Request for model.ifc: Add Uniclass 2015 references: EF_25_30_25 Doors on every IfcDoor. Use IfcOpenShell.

First a look at what the model holds.

```python
import ifcopenshell

model = ifcopenshell.open("model.ifc")
print(model.schema)
print("classifications:", [c.Name for c in model.by_type("IfcClassification")])
for ifc_class in ("IfcDoor", "IfcRoof", "IfcStair", "IfcWall", "IfcWindow"):
    print(ifc_class, len(model.by_type(ifc_class)))
```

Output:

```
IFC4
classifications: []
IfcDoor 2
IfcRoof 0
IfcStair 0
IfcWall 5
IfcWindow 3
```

```python
import ifcopenshell
import ifcopenshell.api.classification

model = ifcopenshell.open("model.ifc")

system = ifcopenshell.api.classification.add_classification(model, classification="Uniclass 2015")

codes = {
    "IfcDoor": ("EF_25_30_25", "Doors"),
}
for ifc_class, (code, name) in codes.items():
    products = model.by_type(ifc_class)
    ifcopenshell.api.classification.add_reference(
        model, products=products, classification=system, identification=code, name=name
    )
    print(code, len(products))

model.write("model_updated.ifc")
```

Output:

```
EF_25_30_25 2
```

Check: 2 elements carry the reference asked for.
